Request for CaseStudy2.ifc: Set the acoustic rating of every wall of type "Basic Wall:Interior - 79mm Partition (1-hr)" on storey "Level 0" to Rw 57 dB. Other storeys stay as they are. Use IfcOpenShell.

First a look at what the model holds.

```python
import ifcopenshell
import ifcopenshell.util.element

model = ifcopenshell.open("CaseStudy2.ifc")
print(model.schema)
storey = next(s for s in model.by_type("IfcBuildingStorey") if s.Name == "Level 0")
walls = [e for e in ifcopenshell.util.element.get_decomposition(storey) if e.is_a("IfcWall")]
seen = {}
for e in walls:
    element_type = ifcopenshell.util.element.get_type(e)
    key = (element_type.Name if element_type != e and element_type else None, ifcopenshell.util.element.get_pset(e, "Pset_WallCommon", "AcousticRating"))
    seen[key] = seen.get(key, 0) + 1
for (name, value), count in sorted(seen.items(), key=str):
    print(count, "x", name, "|", value)
```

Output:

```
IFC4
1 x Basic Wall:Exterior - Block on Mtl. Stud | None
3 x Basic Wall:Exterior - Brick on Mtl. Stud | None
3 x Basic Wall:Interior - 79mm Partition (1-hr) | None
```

```python
import ifcopenshell
import ifcopenshell.api.pset
import ifcopenshell.util.element

model = ifcopenshell.open("CaseStudy2.ifc")

storey = next(s for s in model.by_type("IfcBuildingStorey") if s.Name == "Level 0")
walls = [e for e in ifcopenshell.util.element.get_decomposition(storey) if e.is_a("IfcWall")]

count = 0
for e in walls:
    element_type = ifcopenshell.util.element.get_type(e)
    if element_type in (None, e) or element_type.Name != "Basic Wall:Interior - 79mm Partition (1-hr)":
        continue
    # add_pset returns the element's existing set when there is one.
    pset = ifcopenshell.api.pset.add_pset(model, product=e, name="Pset_WallCommon")
    ifcopenshell.api.pset.edit_pset(model, pset=pset, properties={"AcousticRating": "Rw 57 dB"})
    count += 1

print(count, "walls updated")

model.write("CaseStudy2-out.ifc")
```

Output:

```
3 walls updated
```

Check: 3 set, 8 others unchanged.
